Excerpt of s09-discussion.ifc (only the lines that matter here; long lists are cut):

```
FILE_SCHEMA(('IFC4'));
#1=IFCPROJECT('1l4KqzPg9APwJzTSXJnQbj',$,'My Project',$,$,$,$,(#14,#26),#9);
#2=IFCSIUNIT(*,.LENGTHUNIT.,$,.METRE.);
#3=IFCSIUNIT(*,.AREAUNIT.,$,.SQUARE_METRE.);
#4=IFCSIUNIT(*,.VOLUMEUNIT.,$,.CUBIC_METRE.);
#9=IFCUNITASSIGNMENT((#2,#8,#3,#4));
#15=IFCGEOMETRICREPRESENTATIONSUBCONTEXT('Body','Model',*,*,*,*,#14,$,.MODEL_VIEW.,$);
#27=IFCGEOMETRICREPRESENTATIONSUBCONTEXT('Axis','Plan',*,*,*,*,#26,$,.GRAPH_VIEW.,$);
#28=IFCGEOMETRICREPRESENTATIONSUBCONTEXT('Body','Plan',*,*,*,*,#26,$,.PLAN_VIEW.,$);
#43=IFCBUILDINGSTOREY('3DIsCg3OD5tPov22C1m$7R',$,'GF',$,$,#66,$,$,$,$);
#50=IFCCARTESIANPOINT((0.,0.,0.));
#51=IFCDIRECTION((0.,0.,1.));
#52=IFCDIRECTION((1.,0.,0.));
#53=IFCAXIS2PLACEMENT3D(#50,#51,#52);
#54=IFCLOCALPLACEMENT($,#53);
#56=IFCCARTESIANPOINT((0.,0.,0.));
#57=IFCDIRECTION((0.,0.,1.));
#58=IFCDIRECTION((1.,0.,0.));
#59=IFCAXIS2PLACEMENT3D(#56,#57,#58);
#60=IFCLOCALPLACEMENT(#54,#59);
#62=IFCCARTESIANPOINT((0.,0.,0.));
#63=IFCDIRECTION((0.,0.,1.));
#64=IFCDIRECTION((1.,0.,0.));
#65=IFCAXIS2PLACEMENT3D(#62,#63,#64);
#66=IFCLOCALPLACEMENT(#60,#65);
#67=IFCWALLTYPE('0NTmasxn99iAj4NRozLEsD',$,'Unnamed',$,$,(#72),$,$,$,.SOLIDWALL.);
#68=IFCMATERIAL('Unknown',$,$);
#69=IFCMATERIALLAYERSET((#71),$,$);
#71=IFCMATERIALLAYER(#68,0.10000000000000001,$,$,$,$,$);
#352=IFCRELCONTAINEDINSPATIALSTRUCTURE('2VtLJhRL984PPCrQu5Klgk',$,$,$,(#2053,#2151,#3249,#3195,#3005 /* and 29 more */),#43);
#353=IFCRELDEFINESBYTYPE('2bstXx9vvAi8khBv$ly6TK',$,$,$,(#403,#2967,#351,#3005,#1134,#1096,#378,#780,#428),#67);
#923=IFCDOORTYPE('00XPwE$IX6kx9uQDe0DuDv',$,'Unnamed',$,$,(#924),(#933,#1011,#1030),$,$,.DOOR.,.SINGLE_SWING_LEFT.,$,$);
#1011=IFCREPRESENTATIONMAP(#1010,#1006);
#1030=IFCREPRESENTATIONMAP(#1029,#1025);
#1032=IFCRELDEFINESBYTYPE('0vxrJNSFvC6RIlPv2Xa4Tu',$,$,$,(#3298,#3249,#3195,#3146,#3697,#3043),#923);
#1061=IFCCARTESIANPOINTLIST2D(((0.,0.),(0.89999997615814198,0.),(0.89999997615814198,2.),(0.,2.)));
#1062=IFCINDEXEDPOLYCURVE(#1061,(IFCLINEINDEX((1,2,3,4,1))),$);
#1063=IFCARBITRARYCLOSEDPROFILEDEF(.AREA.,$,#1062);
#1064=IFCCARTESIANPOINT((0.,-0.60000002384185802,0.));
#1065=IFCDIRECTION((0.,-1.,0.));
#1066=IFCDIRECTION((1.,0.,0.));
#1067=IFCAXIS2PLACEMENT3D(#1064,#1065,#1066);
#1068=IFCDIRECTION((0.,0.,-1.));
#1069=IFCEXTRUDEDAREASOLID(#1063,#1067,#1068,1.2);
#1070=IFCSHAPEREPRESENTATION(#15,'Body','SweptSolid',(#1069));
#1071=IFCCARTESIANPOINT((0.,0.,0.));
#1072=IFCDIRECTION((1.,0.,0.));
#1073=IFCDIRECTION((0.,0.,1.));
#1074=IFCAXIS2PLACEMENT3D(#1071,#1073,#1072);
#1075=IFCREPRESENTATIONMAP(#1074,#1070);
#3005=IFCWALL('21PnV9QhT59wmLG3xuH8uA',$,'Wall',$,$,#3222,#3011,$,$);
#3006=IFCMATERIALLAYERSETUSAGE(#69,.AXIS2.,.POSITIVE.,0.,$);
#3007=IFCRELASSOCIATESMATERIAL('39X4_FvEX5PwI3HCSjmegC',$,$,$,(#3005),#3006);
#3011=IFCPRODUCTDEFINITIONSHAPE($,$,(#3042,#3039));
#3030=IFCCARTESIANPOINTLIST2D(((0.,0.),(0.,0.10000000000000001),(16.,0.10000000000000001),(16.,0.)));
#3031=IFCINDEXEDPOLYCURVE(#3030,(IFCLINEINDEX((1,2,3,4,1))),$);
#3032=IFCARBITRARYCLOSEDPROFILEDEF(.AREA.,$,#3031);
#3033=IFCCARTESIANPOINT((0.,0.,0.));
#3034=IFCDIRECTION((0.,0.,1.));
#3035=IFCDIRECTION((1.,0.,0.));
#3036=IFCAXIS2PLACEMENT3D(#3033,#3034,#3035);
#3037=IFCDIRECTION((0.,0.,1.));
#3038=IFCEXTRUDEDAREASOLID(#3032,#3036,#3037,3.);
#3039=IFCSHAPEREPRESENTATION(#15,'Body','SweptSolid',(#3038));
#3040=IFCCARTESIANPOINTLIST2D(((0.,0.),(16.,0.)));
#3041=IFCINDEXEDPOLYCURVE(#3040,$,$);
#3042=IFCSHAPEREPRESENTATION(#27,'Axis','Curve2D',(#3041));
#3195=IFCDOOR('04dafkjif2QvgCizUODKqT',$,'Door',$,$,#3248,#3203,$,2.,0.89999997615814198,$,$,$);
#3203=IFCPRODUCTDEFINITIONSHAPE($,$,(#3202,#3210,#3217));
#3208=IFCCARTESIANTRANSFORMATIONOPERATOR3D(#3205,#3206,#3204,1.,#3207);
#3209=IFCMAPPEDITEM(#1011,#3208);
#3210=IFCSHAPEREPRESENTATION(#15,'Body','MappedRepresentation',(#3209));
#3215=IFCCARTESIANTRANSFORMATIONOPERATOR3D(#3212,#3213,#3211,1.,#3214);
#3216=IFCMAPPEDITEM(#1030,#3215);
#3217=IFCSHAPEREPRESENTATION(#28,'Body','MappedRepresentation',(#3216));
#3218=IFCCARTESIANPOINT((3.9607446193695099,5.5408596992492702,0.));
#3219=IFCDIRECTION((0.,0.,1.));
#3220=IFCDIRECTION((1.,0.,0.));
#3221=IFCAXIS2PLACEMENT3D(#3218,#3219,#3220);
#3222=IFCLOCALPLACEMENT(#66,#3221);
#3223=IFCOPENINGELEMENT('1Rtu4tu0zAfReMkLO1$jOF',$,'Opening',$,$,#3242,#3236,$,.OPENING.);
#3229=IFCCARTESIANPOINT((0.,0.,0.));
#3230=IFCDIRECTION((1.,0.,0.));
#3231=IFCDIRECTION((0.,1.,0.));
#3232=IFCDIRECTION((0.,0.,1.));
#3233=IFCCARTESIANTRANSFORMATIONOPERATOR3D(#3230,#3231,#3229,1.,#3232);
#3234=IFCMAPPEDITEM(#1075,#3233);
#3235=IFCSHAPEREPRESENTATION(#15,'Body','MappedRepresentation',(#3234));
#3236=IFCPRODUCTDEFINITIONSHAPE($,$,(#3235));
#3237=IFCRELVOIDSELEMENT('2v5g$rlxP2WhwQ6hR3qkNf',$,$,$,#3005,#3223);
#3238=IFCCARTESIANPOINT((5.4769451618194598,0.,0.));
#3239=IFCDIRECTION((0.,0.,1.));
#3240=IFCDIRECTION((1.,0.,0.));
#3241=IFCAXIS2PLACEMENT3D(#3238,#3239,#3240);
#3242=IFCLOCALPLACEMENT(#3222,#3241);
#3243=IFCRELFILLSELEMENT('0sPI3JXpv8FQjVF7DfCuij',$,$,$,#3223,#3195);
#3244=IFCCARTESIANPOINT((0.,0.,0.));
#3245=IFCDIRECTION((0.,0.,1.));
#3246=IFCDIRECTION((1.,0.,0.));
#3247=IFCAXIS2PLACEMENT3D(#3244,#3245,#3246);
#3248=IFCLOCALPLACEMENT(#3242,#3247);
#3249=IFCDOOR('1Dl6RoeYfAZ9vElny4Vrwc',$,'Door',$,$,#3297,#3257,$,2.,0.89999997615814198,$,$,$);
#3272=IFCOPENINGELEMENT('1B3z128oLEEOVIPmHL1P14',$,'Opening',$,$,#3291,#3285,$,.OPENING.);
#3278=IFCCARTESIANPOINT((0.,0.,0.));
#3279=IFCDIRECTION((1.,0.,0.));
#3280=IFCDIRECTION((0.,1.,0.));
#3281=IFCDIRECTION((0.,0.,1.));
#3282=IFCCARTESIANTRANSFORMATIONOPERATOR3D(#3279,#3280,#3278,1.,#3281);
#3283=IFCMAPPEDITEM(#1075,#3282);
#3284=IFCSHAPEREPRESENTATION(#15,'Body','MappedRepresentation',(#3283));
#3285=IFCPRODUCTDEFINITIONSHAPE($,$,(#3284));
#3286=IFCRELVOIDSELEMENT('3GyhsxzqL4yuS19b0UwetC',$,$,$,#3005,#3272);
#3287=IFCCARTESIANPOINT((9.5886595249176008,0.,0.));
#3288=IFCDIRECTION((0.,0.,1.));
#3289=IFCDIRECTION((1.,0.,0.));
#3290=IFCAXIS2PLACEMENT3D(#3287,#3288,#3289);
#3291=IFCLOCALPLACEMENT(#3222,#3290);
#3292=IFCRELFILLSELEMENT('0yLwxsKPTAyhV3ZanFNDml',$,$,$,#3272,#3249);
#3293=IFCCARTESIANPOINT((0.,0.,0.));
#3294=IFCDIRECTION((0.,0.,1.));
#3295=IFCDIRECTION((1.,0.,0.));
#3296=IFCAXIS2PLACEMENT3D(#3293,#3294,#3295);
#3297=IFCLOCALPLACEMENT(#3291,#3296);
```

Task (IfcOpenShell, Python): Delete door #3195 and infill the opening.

```python
import ifcopenshell
import ifcopenshell.api.feature
import ifcopenshell.api.root
import ifcopenshell.geom
import ifcopenshell.util.shape

model = ifcopenshell.open("s09-discussion.ifc")
settings = ifcopenshell.geom.settings()


def volume(element):
    """Net volume in cubic metres, openings subtracted."""
    shape = ifcopenshell.geom.create_shape(settings, element)
    return ifcopenshell.util.shape.get_volume(shape.geometry)


door = model.by_id(3195)
opening = door.FillsVoids[0].RelatingOpeningElement
wall = opening.VoidsElements[0].RelatingBuildingElement
before = volume(wall)

ifcopenshell.api.root.remove_product(model, product=door)
ifcopenshell.api.feature.remove_feature(model, feature=opening)

after = volume(wall)

print(f"wall volume {before:.3f} -> {after:.3f} m3")

model.write("s09-discussion_v2.ifc")
```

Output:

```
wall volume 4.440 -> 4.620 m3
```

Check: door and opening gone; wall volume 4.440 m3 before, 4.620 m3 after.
